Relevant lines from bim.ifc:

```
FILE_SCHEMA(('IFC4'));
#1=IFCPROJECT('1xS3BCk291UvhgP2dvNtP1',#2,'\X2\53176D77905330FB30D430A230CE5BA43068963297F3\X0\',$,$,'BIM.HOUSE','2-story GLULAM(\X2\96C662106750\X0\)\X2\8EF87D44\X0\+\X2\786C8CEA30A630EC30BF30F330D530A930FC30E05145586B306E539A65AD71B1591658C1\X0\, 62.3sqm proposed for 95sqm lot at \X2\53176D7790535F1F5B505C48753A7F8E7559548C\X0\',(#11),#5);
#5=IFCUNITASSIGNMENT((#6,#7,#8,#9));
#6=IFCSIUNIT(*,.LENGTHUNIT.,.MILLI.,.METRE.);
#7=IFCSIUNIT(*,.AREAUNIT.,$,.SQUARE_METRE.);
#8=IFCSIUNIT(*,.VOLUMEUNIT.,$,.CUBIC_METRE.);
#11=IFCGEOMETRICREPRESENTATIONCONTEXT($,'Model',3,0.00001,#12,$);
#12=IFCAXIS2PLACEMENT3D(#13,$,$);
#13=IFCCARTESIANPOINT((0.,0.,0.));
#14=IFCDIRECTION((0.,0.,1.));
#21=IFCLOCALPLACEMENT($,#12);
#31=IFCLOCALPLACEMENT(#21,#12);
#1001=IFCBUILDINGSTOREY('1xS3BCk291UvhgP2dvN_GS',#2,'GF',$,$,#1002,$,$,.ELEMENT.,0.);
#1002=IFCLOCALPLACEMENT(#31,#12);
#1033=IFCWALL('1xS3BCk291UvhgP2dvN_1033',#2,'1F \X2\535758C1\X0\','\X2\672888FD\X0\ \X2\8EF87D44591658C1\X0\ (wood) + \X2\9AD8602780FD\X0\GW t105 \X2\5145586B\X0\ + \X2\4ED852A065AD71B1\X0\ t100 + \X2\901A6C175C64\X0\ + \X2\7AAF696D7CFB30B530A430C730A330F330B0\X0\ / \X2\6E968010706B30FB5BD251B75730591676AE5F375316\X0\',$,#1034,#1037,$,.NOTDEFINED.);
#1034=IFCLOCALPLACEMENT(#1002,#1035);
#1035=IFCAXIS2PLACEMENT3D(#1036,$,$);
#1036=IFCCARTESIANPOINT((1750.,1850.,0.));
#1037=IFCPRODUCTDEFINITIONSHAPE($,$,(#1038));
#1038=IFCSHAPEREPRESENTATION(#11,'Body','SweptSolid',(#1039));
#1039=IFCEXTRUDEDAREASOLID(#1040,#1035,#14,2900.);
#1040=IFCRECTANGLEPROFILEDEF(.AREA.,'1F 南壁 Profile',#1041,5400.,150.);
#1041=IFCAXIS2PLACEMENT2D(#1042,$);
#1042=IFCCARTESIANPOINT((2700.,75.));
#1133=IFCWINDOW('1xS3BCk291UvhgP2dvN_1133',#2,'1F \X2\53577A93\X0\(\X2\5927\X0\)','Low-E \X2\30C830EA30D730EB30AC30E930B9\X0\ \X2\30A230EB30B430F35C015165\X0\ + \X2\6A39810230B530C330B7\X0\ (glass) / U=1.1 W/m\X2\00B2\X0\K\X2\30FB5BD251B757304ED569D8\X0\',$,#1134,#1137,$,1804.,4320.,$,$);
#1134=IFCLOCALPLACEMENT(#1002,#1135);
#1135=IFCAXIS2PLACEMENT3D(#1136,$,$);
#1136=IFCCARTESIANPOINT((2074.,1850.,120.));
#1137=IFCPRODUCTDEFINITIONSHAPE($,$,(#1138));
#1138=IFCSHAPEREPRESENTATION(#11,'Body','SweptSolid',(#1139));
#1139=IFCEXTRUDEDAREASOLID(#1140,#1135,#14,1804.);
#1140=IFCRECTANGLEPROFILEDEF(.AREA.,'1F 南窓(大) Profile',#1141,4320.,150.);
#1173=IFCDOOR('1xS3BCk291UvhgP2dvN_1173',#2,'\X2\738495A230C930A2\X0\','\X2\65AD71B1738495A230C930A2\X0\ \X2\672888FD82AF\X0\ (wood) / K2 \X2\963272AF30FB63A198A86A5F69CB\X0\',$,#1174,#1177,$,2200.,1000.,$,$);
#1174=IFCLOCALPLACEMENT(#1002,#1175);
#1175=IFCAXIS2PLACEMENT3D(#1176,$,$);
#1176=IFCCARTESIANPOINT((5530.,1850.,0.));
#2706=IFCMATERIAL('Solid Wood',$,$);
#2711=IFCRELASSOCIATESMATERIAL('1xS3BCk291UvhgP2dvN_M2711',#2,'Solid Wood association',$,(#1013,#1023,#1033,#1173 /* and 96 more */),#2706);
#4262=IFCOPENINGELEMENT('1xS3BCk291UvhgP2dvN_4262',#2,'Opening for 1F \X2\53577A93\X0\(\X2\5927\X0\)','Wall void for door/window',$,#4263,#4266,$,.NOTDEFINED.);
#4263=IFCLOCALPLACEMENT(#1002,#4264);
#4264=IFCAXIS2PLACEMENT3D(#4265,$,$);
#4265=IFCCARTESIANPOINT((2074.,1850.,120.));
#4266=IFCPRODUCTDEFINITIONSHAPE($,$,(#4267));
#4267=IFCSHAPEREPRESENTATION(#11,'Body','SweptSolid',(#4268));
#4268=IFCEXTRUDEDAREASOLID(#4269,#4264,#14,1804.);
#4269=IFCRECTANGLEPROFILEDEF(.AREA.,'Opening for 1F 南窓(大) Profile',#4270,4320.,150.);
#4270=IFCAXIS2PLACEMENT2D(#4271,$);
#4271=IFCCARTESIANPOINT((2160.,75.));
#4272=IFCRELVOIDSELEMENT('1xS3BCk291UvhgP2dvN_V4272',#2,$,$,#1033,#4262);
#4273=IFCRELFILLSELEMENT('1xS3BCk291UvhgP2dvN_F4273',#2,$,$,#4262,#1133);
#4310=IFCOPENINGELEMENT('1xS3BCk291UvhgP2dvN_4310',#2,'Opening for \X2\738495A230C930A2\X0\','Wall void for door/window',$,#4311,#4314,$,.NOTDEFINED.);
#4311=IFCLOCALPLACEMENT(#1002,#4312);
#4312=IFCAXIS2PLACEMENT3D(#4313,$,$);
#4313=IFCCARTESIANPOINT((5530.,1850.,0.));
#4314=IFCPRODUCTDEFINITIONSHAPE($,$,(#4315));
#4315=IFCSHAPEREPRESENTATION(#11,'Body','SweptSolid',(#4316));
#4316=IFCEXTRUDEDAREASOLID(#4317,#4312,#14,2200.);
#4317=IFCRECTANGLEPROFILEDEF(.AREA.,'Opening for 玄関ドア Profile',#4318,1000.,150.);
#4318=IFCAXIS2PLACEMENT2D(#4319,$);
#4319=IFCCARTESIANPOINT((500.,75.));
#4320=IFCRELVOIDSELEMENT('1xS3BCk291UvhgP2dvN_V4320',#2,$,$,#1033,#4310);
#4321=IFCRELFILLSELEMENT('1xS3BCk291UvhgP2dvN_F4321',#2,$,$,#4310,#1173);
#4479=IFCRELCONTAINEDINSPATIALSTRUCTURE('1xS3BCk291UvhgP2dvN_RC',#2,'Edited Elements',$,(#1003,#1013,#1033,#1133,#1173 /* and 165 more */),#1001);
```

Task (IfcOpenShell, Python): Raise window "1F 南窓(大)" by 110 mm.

```python
import numpy as np
import ifcopenshell
import ifcopenshell.api.geometry
import ifcopenshell.util.placement
import ifcopenshell.util.unit

model = ifcopenshell.open("bim.ifc")
unit_scale = ifcopenshell.util.unit.calculate_unit_scale(model)

window = model.by_id(1133)
opening = window.FillsVoids[0].RelatingOpeningElement
dz = 0.11 / unit_scale

shift = np.array([0.0, 0.0, dz])
# The window is not placed relative to its opening, so move both.
for product in (opening, window):
    matrix = ifcopenshell.util.placement.get_local_placement(product.ObjectPlacement)
    matrix[:3, 3] += shift
    ifcopenshell.api.geometry.edit_object_placement(model, product=product, matrix=matrix, is_si=False)

print(f"moved by {dz * unit_scale:+.3f} m")

model.write("bim_updated.ifc")
```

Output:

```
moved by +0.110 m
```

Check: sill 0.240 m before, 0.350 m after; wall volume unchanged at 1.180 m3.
